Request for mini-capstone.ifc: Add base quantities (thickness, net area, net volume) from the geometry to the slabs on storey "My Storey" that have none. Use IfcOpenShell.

First a look at what the model holds.

```python
import ifcopenshell
import ifcopenshell.util.element
import ifcopenshell.util.unit

model = ifcopenshell.open("mini-capstone.ifc")
print(model.schema)
for unit_type in ("LENGTHUNIT", "AREAUNIT", "VOLUMEUNIT"):
    print(unit_type, ifcopenshell.util.unit.calculate_unit_scale(model, unit_type))
storey = next(s for s in model.by_type("IfcBuildingStorey") if s.Name == "My Storey")
slabs = [e for e in ifcopenshell.util.element.get_decomposition(storey) if e.is_a("IfcSlab")]
for e in sorted(slabs, key=lambda e: e.id()):
    print(e.id(), e.is_a(), e.Name, list(ifcopenshell.util.element.get_psets(e, qtos_only=True)), sep=" | ")
```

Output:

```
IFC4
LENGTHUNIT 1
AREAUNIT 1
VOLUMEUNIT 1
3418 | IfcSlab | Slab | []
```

```python
import ifcopenshell
import ifcopenshell.api.pset
import ifcopenshell.geom
import ifcopenshell.util.element
import ifcopenshell.util.shape
import ifcopenshell.util.unit

model = ifcopenshell.open("mini-capstone.ifc")
unit_scale = ifcopenshell.util.unit.calculate_unit_scale(model)
area_scale = ifcopenshell.util.unit.calculate_unit_scale(model, "AREAUNIT")
volume_scale = ifcopenshell.util.unit.calculate_unit_scale(model, "VOLUMEUNIT")
settings = ifcopenshell.geom.settings()

storey = next(s for s in model.by_type("IfcBuildingStorey") if s.Name == "My Storey")
slabs = [e for e in ifcopenshell.util.element.get_decomposition(storey) if e.is_a("IfcSlab")]

for e in sorted(slabs, key=lambda e: e.id()):
    if ifcopenshell.util.element.get_psets(e, qtos_only=True, should_inherit=False):
        continue
    # Geometry comes back in metres, in the element's own axes.
    shape = ifcopenshell.geom.create_shape(settings, e)
    values = {
        "Width": ifcopenshell.util.shape.get_z(shape.geometry) / unit_scale,
        "NetArea": ifcopenshell.util.shape.get_footprint_area(shape.geometry) / area_scale,
        "NetVolume": ifcopenshell.util.shape.get_volume(shape.geometry) / volume_scale,
    }
    qto = ifcopenshell.api.pset.add_qto(model, product=e, name="Qto_SlabBaseQuantities")
    ifcopenshell.api.pset.edit_qto(model, qto=qto, properties=values)
    print(e.id(), {k: round(v, 3) for k, v in values.items()})

model.write("mini-capstone-out.ifc")
```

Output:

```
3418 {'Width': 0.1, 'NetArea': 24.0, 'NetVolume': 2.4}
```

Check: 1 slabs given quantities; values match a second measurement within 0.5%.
